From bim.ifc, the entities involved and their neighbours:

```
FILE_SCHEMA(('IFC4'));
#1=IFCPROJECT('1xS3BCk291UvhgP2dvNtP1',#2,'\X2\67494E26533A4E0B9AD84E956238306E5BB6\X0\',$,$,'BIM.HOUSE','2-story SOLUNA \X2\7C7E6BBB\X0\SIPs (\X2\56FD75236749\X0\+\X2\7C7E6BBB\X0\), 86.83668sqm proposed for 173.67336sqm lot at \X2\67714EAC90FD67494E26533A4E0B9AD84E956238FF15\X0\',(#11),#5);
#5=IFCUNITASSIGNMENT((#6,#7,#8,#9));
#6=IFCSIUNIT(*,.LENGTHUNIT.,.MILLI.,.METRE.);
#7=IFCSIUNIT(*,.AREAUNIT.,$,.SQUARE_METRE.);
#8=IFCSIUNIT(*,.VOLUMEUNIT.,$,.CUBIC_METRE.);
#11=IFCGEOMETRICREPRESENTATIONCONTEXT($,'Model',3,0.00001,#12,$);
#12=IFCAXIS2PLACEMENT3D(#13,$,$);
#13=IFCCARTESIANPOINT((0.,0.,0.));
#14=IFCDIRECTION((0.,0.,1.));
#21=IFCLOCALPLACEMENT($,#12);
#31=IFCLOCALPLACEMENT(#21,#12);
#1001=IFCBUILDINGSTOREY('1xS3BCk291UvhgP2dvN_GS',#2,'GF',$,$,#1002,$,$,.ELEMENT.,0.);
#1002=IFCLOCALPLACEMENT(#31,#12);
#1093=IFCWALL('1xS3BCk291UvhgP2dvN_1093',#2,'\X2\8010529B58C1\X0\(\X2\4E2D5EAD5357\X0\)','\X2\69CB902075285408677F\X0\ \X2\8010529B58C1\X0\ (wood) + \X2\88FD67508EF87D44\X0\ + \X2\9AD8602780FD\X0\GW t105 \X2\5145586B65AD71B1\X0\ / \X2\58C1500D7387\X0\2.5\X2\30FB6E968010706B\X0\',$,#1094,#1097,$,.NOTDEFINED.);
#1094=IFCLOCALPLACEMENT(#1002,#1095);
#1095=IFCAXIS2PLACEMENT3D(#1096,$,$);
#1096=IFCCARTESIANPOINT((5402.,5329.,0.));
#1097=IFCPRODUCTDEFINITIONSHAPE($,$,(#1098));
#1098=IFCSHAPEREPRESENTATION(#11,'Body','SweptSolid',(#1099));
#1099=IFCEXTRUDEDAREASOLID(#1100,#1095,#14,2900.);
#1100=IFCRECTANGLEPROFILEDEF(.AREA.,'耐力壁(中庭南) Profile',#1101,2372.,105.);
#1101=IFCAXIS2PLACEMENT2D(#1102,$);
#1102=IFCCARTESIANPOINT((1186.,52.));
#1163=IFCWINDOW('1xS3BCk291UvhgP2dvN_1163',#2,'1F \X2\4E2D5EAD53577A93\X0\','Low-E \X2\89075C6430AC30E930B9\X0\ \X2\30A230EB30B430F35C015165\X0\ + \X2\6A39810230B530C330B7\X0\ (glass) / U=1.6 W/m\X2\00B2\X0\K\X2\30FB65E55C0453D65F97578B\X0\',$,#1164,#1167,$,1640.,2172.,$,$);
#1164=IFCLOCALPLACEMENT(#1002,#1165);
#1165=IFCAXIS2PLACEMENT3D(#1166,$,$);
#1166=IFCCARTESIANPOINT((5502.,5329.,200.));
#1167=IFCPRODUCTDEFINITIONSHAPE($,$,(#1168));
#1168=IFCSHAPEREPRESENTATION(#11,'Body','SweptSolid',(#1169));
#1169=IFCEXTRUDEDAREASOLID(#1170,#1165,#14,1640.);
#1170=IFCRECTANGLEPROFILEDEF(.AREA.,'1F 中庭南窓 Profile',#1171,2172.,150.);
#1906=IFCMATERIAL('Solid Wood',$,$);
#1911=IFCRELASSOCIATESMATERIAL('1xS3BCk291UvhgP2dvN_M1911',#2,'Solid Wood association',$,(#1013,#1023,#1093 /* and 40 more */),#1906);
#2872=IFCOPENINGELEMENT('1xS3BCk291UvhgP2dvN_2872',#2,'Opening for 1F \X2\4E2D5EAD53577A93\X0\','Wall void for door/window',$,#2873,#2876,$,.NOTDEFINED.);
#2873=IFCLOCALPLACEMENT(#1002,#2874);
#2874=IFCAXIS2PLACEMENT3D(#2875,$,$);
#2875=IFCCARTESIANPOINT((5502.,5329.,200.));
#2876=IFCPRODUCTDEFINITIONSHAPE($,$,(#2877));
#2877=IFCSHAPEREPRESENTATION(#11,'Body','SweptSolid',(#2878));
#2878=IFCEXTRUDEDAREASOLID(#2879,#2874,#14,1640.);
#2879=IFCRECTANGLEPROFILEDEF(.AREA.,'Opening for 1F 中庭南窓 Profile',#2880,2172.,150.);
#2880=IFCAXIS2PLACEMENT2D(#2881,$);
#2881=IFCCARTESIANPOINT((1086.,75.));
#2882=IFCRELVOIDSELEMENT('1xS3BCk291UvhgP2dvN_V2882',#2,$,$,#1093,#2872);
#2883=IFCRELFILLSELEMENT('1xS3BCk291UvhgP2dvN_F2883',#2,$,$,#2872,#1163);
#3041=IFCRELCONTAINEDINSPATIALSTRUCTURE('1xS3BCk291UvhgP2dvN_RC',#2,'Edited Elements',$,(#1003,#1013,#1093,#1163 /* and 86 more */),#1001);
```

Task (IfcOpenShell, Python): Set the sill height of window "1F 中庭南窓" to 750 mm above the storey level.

```python
import numpy as np
import ifcopenshell
import ifcopenshell.api.geometry
import ifcopenshell.geom
import ifcopenshell.util.element
import ifcopenshell.util.placement
import ifcopenshell.util.shape
import ifcopenshell.util.unit

model = ifcopenshell.open("bim.ifc")
unit_scale = ifcopenshell.util.unit.calculate_unit_scale(model)

window = model.by_id(1163)
opening = window.FillsVoids[0].RelatingOpeningElement
storey = ifcopenshell.util.element.get_container(window, ifc_class="IfcBuildingStorey")
level = ifcopenshell.util.placement.get_local_placement(storey.ObjectPlacement)[2, 3]

# The opening's origin need not be at the sill, so measure its lowest point.
shape = ifcopenshell.geom.create_shape(ifcopenshell.geom.settings(), opening)
bottom = ifcopenshell.util.shape.get_shape_bottom_elevation(shape, shape.geometry) / unit_scale
dz = level + 0.75 / unit_scale - bottom

shift = np.array([0.0, 0.0, dz])
# The window is not placed relative to its opening, so move both.
for product in (opening, window):
    matrix = ifcopenshell.util.placement.get_local_placement(product.ObjectPlacement)
    matrix[:3, 3] += shift
    ifcopenshell.api.geometry.edit_object_placement(model, product=product, matrix=matrix, is_si=False)

print(f"moved by {dz * unit_scale:+.3f} m")

model.write("bim_updated.ifc")
```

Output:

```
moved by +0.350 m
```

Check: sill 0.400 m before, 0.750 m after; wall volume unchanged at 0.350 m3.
